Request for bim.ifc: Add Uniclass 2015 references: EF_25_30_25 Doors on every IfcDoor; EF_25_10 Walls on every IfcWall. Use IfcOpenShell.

First a look at what the model holds.

```python
import ifcopenshell

model = ifcopenshell.open("bim.ifc")
print(model.schema)
print("classifications:", [c.Name for c in model.by_type("IfcClassification")])
for ifc_class in ("IfcDoor", "IfcRoof", "IfcStair", "IfcWall", "IfcWindow"):
    print(ifc_class, len(model.by_type(ifc_class)))
```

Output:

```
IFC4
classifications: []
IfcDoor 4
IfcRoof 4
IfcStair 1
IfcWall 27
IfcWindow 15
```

```python
import ifcopenshell
import ifcopenshell.api.classification

model = ifcopenshell.open("bim.ifc")

system = ifcopenshell.api.classification.add_classification(model, classification="Uniclass 2015")

codes = {
    "IfcDoor": ("EF_25_30_25", "Doors"),
    "IfcWall": ("EF_25_10", "Walls"),
}
for ifc_class, (code, name) in codes.items():
    products = model.by_type(ifc_class)
    ifcopenshell.api.classification.add_reference(
        model, products=products, classification=system, identification=code, name=name
    )
    print(code, len(products))

model.write("bim_edited.ifc")
```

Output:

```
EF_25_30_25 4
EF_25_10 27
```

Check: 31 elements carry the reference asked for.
